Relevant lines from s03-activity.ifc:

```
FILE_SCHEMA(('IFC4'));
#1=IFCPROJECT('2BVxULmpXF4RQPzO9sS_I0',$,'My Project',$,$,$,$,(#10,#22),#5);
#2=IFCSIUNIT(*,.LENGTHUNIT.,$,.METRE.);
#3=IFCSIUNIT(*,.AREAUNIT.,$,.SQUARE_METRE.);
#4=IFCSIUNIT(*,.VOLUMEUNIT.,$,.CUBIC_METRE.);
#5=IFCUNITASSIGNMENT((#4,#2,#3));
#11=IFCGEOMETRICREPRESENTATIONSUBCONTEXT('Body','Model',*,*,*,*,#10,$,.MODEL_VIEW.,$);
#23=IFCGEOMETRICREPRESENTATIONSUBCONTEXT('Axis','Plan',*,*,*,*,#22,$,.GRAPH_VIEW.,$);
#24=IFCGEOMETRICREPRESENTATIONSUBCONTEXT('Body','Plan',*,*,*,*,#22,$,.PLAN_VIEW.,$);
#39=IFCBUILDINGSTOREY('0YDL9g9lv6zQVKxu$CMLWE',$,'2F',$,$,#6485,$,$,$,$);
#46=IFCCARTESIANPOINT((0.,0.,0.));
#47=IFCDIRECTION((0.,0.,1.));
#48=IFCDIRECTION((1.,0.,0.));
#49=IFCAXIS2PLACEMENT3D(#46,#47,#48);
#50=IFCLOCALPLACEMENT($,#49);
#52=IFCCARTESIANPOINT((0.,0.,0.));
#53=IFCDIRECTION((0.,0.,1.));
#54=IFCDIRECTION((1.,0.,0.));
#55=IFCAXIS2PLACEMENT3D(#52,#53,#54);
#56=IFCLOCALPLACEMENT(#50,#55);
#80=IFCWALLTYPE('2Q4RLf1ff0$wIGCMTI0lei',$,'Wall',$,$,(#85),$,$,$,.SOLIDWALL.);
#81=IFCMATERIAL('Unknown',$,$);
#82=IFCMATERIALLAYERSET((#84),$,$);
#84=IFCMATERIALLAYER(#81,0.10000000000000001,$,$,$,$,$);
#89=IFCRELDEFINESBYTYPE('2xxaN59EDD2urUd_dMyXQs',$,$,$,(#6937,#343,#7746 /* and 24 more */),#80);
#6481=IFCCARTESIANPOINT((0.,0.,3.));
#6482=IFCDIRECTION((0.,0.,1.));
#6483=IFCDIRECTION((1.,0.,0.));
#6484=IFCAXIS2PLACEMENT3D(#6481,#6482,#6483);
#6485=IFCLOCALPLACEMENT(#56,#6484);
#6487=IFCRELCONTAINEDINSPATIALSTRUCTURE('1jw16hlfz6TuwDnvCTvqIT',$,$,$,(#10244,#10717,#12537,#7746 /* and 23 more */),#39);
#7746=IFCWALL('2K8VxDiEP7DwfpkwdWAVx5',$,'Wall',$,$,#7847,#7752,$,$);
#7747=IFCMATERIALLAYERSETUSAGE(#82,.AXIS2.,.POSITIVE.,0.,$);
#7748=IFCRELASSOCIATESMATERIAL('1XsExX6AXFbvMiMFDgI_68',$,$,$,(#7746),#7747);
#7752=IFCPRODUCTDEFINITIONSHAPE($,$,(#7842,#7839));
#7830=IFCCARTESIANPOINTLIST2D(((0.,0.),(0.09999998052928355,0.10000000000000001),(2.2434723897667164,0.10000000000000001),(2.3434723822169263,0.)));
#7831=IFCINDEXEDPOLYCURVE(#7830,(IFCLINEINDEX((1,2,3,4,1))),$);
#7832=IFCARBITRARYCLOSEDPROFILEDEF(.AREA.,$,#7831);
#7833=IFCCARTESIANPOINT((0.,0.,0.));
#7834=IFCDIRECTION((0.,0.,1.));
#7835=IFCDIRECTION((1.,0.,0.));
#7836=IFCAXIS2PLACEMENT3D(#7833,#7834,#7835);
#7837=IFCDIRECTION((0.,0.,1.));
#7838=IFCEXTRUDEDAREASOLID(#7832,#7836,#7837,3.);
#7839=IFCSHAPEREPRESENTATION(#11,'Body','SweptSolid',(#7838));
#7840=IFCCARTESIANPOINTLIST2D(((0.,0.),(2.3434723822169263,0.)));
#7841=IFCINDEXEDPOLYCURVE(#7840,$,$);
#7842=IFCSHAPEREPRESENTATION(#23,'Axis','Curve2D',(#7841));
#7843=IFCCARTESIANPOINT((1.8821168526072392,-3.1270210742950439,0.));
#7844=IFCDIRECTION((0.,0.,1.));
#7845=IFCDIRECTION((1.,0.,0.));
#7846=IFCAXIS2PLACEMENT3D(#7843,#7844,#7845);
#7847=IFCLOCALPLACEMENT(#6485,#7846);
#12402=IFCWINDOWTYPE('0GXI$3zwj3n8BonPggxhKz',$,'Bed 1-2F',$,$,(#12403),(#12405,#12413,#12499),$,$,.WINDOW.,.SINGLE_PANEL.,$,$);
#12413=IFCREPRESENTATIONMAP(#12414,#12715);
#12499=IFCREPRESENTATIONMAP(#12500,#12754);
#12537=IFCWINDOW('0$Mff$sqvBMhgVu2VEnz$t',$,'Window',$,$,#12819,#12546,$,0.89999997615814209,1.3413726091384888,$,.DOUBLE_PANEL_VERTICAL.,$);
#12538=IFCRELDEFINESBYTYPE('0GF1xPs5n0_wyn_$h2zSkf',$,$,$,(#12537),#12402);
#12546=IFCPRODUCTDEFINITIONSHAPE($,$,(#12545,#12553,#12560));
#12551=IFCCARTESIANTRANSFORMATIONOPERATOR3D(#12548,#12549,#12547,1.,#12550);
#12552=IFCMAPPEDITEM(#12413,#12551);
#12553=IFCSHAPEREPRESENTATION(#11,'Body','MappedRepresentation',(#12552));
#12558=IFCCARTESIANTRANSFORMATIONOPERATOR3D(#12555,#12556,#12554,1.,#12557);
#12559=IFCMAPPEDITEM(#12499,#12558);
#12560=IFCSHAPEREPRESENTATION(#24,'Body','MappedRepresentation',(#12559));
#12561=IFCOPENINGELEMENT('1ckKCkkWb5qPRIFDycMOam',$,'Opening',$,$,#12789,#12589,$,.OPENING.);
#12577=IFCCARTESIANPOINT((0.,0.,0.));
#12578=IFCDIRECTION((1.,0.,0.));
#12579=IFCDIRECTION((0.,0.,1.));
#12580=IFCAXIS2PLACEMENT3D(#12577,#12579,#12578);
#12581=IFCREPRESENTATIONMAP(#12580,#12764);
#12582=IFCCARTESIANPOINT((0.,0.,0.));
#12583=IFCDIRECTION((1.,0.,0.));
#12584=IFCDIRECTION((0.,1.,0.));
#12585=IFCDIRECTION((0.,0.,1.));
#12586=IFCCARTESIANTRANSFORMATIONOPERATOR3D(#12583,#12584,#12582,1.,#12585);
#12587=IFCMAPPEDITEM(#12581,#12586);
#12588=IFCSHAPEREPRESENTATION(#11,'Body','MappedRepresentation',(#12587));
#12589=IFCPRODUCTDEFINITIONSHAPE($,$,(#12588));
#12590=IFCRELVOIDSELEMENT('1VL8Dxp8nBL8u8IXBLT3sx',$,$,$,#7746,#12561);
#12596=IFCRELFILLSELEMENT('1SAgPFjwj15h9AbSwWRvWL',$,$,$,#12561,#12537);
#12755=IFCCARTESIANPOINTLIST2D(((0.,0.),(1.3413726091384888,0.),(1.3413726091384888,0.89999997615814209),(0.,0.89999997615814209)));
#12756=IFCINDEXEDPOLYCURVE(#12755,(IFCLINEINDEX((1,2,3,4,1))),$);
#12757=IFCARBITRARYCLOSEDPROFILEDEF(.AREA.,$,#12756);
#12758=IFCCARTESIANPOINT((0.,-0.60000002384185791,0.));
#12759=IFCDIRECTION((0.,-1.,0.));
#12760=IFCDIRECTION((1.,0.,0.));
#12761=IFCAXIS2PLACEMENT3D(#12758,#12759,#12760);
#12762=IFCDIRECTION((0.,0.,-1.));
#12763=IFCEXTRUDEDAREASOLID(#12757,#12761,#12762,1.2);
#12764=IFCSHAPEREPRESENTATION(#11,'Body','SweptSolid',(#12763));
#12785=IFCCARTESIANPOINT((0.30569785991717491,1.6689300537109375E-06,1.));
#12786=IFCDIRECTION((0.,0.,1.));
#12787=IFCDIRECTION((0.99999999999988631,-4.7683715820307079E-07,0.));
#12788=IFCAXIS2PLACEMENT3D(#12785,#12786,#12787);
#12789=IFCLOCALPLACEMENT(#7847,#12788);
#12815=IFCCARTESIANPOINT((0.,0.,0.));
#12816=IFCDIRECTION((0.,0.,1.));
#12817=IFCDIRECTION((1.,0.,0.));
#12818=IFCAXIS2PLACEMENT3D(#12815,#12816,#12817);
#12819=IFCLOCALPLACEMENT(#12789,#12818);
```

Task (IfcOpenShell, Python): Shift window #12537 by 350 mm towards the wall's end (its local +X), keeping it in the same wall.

```python
import ifcopenshell
import ifcopenshell.api.geometry
import ifcopenshell.util.placement
import ifcopenshell.util.unit

model = ifcopenshell.open("s03-activity.ifc")
unit_scale = ifcopenshell.util.unit.calculate_unit_scale(model)

window = model.by_id(12537)
opening = window.FillsVoids[0].RelatingOpeningElement
wall = opening.VoidsElements[0].RelatingBuildingElement

wall_matrix = ifcopenshell.util.placement.get_local_placement(wall.ObjectPlacement)
shift = wall_matrix[:3, 0] * 0.35 / unit_scale
before = ifcopenshell.util.placement.get_local_placement(window.ObjectPlacement)[:3, 3].copy()

# The window is placed relative to its opening, so it follows when the opening moves.
matrix = ifcopenshell.util.placement.get_local_placement(opening.ObjectPlacement)
matrix[:3, 3] += shift
ifcopenshell.api.geometry.edit_object_placement(
    model, product=opening, matrix=matrix, is_si=False, should_transform_children=True
)

after = ifcopenshell.util.placement.get_local_placement(window.ObjectPlacement)[:3, 3]
print("window moved by", (after - before).round(3) + 0.0)

model.write("s03-activity_rev.ifc")
```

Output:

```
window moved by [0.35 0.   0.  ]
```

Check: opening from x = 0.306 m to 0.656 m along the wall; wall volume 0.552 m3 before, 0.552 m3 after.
